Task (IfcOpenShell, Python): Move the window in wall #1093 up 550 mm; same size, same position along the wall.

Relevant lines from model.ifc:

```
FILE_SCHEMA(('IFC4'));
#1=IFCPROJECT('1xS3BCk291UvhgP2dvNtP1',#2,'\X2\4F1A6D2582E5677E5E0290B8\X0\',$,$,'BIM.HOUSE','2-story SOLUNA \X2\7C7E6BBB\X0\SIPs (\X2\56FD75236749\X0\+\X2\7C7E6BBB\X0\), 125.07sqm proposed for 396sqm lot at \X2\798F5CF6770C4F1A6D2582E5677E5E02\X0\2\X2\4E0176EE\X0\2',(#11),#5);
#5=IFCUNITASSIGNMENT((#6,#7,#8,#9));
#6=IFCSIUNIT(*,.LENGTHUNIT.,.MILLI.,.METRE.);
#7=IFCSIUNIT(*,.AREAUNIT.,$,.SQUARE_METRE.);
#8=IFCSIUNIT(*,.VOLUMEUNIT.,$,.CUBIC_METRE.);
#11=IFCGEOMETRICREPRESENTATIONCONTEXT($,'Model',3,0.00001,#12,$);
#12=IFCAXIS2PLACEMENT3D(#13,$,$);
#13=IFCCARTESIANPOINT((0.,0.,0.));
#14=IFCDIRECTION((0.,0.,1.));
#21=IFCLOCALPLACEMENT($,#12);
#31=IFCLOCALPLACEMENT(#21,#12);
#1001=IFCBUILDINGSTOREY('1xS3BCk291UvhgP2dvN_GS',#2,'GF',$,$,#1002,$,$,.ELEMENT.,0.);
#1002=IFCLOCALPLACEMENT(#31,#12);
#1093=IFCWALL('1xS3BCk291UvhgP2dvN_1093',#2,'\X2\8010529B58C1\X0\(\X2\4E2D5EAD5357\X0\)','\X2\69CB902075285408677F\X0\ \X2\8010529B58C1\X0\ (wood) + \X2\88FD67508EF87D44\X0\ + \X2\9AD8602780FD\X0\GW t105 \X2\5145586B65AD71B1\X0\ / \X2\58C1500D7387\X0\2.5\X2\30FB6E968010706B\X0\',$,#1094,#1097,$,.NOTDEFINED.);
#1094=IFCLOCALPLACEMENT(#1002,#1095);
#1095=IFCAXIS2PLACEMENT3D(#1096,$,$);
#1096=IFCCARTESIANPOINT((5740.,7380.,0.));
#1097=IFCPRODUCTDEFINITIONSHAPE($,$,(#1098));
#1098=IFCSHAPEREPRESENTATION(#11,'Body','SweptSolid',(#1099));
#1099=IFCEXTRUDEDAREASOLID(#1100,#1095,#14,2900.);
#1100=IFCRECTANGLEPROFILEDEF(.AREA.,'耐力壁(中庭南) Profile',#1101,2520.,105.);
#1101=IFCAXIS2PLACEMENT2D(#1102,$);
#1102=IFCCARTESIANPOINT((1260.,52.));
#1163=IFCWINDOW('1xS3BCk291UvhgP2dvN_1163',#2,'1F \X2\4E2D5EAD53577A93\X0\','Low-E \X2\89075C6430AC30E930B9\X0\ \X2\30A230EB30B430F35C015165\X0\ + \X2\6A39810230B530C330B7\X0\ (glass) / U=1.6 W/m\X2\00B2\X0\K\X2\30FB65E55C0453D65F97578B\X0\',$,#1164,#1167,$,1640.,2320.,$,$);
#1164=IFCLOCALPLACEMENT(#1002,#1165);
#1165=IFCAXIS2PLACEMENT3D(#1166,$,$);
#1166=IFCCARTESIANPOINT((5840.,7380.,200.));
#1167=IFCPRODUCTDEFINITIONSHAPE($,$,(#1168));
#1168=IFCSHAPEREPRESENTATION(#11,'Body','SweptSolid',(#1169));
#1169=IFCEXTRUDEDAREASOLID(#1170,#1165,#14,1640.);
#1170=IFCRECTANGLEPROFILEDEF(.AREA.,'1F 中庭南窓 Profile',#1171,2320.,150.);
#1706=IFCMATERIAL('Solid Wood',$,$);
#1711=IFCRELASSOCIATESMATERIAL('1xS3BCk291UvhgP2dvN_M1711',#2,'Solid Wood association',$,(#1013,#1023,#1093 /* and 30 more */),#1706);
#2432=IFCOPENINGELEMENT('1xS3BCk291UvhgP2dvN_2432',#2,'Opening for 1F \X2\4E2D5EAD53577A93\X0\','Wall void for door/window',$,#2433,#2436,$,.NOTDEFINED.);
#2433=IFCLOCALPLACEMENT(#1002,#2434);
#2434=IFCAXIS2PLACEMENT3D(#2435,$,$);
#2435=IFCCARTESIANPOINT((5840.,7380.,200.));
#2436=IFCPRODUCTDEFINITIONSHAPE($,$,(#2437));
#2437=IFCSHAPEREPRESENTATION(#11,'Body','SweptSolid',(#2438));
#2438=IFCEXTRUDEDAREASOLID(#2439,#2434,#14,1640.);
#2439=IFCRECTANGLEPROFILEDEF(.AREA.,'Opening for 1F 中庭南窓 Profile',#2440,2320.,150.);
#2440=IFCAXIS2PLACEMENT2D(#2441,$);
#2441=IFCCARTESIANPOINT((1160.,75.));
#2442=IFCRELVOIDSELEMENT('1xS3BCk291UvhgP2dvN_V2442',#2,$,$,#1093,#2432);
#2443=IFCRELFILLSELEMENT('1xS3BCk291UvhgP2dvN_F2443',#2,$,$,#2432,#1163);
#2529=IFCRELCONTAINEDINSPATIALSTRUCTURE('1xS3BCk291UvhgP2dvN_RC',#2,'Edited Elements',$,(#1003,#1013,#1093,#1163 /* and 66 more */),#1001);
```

```python
import numpy as np
import ifcopenshell
import ifcopenshell.api.geometry
import ifcopenshell.util.placement
import ifcopenshell.util.unit

model = ifcopenshell.open("model.ifc")
unit_scale = ifcopenshell.util.unit.calculate_unit_scale(model)

window = model.by_guid("1xS3BCk291UvhgP2dvN_1163")
opening = window.FillsVoids[0].RelatingOpeningElement
dz = 550.0

shift = np.array([0.0, 0.0, dz])
# The window is not placed relative to its opening, so move both.
for product in (opening, window):
    matrix = ifcopenshell.util.placement.get_local_placement(product.ObjectPlacement)
    matrix[:3, 3] += shift
    ifcopenshell.api.geometry.edit_object_placement(model, product=product, matrix=matrix, is_si=False)

print(f"moved by {dz * unit_scale:+.3f} m")

model.write("model_updated.ifc")
```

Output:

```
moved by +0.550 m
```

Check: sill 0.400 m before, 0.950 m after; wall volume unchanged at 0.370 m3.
